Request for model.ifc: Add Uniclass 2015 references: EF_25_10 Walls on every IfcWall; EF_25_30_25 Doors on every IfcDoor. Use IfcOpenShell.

First a look at what the model holds.

```python
import ifcopenshell

model = ifcopenshell.open("model.ifc")
print(model.schema)
print("classifications:", [c.Name for c in model.by_type("IfcClassification")])
for ifc_class in ("IfcDoor", "IfcRoof", "IfcStair", "IfcWall", "IfcWindow"):
    print(ifc_class, len(model.by_type(ifc_class)))
```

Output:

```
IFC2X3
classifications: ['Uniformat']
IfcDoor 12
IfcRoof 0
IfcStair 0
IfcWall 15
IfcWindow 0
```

```python
import ifcopenshell
import ifcopenshell.api.classification

model = ifcopenshell.open("model.ifc")

# IFC2X3 requires Source and Edition and has no link from the project to the system.
system = model.create_entity("IfcClassification", Source="NBS", Edition="2015", Name="Uniclass 2015")

codes = {
    "IfcWall": ("EF_25_10", "Walls"),
    "IfcDoor": ("EF_25_30_25", "Doors"),
}
for ifc_class, (code, name) in codes.items():
    products = model.by_type(ifc_class)
    ifcopenshell.api.classification.add_reference(
        model, products=products, classification=system, identification=code, name=name
    )
    print(code, len(products))

model.write("model-out.ifc")
```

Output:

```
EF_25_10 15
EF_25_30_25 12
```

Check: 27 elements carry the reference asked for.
